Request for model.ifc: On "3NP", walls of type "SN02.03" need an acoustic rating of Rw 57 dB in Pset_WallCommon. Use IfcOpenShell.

First a look at what the model holds.

```python
import ifcopenshell
import ifcopenshell.util.element

model = ifcopenshell.open("model.ifc")
print(model.schema)
storey = next(s for s in model.by_type("IfcBuildingStorey") if s.Name == "3NP")
walls = [e for e in ifcopenshell.util.element.get_decomposition(storey) if e.is_a("IfcWall")]
seen = {}
for e in walls:
    element_type = ifcopenshell.util.element.get_type(e)
    key = (element_type.Name if element_type != e and element_type else None, ifcopenshell.util.element.get_pset(e, "Pset_WallCommon", "AcousticRating"))
    seen[key] = seen.get(key, 0) + 1
for (name, value), count in sorted(seen.items(), key=str):
    print(count, "x", name, "|", value)
```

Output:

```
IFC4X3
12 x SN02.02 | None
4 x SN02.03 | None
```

```python
import ifcopenshell
import ifcopenshell.api.pset
import ifcopenshell.util.element

model = ifcopenshell.open("model.ifc")

storey = next(s for s in model.by_type("IfcBuildingStorey") if s.Name == "3NP")
walls = [e for e in ifcopenshell.util.element.get_decomposition(storey) if e.is_a("IfcWall")]

count = 0
for e in walls:
    element_type = ifcopenshell.util.element.get_type(e)
    if element_type in (None, e) or element_type.Name != "SN02.03":
        continue
    # add_pset returns the element's existing set when there is one.
    pset = ifcopenshell.api.pset.add_pset(model, product=e, name="Pset_WallCommon")
    ifcopenshell.api.pset.edit_pset(model, pset=pset, properties={"AcousticRating": "Rw 57 dB"})
    count += 1

print(count, "walls updated")

model.write("model-out.ifc")
```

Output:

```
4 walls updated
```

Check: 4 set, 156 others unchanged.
